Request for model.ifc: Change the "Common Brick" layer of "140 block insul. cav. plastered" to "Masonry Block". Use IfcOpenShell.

First a look at what the model holds.

```python
import ifcopenshell
import ifcopenshell.util.element

model = ifcopenshell.open("model.ifc")
print(model.schema)
for layer_set in model.by_type("IfcMaterialLayerSet"):
    if layer_set.LayerSetName == "140 block insul. cav. plastered":
        for layer in layer_set.MaterialLayers:
            print(layer.id(), layer.Material and layer.Material.Name, layer.LayerThickness, sep=" | ")
        print(len(ifcopenshell.util.element.get_elements_by_material(model, layer_set)), "elements and types use it")
print(sorted(m.Name for m in model.by_type("IfcMaterial") if m.Name)[:60])
```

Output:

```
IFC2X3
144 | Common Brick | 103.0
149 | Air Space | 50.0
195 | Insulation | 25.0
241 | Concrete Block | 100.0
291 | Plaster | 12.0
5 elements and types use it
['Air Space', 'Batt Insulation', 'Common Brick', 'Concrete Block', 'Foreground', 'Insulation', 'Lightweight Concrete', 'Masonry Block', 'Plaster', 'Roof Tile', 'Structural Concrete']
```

```python
import ifcopenshell
import ifcopenshell.api.material

model = ifcopenshell.open("model.ifc")

layer_set = next(s for s in model.by_type("IfcMaterialLayerSet") if s.LayerSetName == "140 block insul. cav. plastered")
layer = next(l for l in layer_set.MaterialLayers if l.Material and l.Material.Name == "Common Brick")
material = next(m for m in model.by_type("IfcMaterial") if m.Name == "Masonry Block")

# Point this one layer at the other material; renaming the old one would change it everywhere.
ifcopenshell.api.material.edit_layer(model, layer=layer, attributes={}, material=material)

print([l.Material.Name if l.Material else None for l in layer_set.MaterialLayers])

model.write("model_edited.ifc")
```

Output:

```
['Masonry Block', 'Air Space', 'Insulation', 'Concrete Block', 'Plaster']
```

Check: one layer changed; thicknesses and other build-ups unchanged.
